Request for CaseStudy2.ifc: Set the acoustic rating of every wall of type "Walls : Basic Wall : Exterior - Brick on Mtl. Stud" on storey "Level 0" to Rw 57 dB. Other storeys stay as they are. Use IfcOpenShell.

First a look at what the model holds.

```python
import ifcopenshell
import ifcopenshell.util.element

model = ifcopenshell.open("CaseStudy2.ifc")
print(model.schema)
storey = next(s for s in model.by_type("IfcBuildingStorey") if s.Name == "Level 0")
walls = [e for e in ifcopenshell.util.element.get_decomposition(storey) if e.is_a("IfcWall")]
seen = {}
for e in walls:
    element_type = ifcopenshell.util.element.get_type(e)
    key = (element_type.Name if element_type != e and element_type else None, ifcopenshell.util.element.get_pset(e, "Pset_WallCommon", "AcousticRating"))
    seen[key] = seen.get(key, 0) + 1
for (name, value), count in sorted(seen.items(), key=str):
    print(count, "x", name, "|", value)
```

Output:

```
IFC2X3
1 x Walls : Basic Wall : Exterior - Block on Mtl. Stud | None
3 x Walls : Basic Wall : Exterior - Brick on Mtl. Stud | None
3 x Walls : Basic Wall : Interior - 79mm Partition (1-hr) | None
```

```python
import ifcopenshell
import ifcopenshell.api.pset
import ifcopenshell.util.element

model = ifcopenshell.open("CaseStudy2.ifc")

storey = next(s for s in model.by_type("IfcBuildingStorey") if s.Name == "Level 0")
walls = [e for e in ifcopenshell.util.element.get_decomposition(storey) if e.is_a("IfcWall")]

count = 0
for e in walls:
    element_type = ifcopenshell.util.element.get_type(e)
    if element_type in (None, e) or element_type.Name != "Walls : Basic Wall : Exterior - Brick on Mtl. Stud":
        continue
    # add_pset returns the element's existing set when there is one.
    pset = ifcopenshell.api.pset.add_pset(model, product=e, name="Pset_WallCommon")
    ifcopenshell.api.pset.edit_pset(model, pset=pset, properties={"AcousticRating": "Rw 57 dB"})
    count += 1

print(count, "walls updated")

model.write("CaseStudy2_rev.ifc")
```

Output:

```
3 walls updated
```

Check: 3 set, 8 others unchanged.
